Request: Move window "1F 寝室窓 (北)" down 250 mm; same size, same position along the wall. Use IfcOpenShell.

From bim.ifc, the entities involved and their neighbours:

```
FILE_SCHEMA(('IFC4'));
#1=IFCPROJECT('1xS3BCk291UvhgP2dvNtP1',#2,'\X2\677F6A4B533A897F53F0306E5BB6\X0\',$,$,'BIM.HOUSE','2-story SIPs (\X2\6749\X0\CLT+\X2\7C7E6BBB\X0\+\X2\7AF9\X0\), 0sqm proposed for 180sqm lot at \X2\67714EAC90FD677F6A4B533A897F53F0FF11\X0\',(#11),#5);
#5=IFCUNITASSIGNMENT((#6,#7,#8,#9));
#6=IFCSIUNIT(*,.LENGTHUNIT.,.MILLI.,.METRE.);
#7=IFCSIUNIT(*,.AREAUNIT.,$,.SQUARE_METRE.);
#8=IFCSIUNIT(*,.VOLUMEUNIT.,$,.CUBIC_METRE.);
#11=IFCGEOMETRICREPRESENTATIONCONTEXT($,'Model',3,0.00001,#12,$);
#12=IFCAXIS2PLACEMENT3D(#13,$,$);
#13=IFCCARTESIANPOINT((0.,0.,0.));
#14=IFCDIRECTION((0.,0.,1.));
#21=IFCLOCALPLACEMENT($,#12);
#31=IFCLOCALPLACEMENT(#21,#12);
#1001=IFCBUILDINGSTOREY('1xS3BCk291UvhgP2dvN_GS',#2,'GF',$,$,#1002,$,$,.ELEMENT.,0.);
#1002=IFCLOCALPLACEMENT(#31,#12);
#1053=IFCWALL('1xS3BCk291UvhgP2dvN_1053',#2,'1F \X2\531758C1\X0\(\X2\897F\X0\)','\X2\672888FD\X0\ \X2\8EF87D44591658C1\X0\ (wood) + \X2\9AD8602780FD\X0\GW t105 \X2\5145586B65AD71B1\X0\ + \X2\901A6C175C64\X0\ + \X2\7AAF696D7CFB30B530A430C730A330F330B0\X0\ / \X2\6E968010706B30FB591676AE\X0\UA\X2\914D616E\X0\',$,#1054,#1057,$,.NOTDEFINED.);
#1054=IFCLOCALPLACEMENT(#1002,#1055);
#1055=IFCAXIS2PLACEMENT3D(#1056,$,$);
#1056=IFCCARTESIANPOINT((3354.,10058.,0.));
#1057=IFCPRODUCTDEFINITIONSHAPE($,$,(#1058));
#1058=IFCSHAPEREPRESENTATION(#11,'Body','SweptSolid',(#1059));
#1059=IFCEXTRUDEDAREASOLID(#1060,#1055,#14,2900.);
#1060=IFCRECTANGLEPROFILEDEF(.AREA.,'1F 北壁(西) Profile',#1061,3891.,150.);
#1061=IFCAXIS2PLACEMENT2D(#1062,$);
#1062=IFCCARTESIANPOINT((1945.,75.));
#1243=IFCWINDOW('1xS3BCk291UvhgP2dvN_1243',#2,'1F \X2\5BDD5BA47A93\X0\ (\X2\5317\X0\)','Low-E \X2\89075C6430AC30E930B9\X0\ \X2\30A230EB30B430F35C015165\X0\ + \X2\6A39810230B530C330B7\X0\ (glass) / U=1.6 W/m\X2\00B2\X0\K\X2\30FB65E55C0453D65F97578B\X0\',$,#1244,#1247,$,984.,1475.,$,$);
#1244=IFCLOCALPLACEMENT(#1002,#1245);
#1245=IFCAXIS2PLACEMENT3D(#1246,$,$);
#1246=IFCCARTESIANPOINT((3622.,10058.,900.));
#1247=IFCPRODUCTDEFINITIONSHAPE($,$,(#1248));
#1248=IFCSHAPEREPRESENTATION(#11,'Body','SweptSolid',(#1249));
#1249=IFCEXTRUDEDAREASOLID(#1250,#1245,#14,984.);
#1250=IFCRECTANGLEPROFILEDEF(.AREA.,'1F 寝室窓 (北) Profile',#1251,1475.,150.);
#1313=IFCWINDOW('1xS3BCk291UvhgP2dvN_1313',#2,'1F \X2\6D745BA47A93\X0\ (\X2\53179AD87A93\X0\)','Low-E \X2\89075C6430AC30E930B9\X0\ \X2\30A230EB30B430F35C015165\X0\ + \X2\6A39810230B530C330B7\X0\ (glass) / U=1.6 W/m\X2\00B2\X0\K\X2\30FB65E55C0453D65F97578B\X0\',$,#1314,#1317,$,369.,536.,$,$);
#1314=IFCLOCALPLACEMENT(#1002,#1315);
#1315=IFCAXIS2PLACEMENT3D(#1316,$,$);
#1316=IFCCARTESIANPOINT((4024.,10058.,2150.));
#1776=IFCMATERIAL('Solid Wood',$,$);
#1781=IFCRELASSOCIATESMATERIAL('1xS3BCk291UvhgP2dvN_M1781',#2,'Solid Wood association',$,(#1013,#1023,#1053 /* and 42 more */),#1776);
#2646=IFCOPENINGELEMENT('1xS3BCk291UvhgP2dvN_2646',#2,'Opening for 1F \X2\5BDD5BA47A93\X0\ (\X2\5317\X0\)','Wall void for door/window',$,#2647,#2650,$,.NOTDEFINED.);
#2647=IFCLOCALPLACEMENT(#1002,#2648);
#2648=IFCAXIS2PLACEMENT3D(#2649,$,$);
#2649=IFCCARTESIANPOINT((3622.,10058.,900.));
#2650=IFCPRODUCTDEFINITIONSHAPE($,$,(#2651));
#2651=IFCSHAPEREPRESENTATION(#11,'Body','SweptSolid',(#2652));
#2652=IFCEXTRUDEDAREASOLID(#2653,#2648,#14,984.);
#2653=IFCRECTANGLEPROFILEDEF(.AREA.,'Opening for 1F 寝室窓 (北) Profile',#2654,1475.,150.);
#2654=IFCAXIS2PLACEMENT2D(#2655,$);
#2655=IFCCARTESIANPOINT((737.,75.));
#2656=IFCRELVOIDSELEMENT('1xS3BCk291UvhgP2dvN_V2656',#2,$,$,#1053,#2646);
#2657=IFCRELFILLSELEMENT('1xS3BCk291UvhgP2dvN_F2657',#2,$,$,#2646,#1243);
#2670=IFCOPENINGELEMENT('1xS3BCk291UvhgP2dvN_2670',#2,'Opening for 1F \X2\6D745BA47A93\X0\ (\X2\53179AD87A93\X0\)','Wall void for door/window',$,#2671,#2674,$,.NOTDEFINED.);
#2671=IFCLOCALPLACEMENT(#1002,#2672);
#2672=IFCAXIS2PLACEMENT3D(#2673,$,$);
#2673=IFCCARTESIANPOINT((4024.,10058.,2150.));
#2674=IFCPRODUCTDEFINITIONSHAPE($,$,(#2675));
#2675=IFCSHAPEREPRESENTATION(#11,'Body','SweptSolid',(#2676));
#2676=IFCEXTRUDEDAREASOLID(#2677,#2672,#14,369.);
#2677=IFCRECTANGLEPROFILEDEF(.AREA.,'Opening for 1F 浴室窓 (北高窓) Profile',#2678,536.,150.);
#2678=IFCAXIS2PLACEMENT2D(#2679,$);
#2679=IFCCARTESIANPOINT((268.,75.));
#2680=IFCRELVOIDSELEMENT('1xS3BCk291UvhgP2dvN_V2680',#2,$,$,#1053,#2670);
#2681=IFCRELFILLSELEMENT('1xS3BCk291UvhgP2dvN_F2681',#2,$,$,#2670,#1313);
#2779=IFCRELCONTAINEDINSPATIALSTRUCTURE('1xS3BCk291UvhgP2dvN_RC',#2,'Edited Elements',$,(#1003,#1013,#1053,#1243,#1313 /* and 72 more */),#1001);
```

```python
import numpy as np
import ifcopenshell
import ifcopenshell.api.geometry
import ifcopenshell.util.placement
import ifcopenshell.util.unit

model = ifcopenshell.open("bim.ifc")
unit_scale = ifcopenshell.util.unit.calculate_unit_scale(model)

window = model.by_guid("1xS3BCk291UvhgP2dvN_1243")
opening = window.FillsVoids[0].RelatingOpeningElement
dz = -0.25 / unit_scale

shift = np.array([0.0, 0.0, dz])
# The window is not placed relative to its opening, so move both.
for product in (opening, window):
    matrix = ifcopenshell.util.placement.get_local_placement(product.ObjectPlacement)
    matrix[:3, 3] += shift
    ifcopenshell.api.geometry.edit_object_placement(model, product=product, matrix=matrix, is_si=False)

print(f"moved by {dz * unit_scale:+.3f} m")

model.write("bim-out.ifc")
```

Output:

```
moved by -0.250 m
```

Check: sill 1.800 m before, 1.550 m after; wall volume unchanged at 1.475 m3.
